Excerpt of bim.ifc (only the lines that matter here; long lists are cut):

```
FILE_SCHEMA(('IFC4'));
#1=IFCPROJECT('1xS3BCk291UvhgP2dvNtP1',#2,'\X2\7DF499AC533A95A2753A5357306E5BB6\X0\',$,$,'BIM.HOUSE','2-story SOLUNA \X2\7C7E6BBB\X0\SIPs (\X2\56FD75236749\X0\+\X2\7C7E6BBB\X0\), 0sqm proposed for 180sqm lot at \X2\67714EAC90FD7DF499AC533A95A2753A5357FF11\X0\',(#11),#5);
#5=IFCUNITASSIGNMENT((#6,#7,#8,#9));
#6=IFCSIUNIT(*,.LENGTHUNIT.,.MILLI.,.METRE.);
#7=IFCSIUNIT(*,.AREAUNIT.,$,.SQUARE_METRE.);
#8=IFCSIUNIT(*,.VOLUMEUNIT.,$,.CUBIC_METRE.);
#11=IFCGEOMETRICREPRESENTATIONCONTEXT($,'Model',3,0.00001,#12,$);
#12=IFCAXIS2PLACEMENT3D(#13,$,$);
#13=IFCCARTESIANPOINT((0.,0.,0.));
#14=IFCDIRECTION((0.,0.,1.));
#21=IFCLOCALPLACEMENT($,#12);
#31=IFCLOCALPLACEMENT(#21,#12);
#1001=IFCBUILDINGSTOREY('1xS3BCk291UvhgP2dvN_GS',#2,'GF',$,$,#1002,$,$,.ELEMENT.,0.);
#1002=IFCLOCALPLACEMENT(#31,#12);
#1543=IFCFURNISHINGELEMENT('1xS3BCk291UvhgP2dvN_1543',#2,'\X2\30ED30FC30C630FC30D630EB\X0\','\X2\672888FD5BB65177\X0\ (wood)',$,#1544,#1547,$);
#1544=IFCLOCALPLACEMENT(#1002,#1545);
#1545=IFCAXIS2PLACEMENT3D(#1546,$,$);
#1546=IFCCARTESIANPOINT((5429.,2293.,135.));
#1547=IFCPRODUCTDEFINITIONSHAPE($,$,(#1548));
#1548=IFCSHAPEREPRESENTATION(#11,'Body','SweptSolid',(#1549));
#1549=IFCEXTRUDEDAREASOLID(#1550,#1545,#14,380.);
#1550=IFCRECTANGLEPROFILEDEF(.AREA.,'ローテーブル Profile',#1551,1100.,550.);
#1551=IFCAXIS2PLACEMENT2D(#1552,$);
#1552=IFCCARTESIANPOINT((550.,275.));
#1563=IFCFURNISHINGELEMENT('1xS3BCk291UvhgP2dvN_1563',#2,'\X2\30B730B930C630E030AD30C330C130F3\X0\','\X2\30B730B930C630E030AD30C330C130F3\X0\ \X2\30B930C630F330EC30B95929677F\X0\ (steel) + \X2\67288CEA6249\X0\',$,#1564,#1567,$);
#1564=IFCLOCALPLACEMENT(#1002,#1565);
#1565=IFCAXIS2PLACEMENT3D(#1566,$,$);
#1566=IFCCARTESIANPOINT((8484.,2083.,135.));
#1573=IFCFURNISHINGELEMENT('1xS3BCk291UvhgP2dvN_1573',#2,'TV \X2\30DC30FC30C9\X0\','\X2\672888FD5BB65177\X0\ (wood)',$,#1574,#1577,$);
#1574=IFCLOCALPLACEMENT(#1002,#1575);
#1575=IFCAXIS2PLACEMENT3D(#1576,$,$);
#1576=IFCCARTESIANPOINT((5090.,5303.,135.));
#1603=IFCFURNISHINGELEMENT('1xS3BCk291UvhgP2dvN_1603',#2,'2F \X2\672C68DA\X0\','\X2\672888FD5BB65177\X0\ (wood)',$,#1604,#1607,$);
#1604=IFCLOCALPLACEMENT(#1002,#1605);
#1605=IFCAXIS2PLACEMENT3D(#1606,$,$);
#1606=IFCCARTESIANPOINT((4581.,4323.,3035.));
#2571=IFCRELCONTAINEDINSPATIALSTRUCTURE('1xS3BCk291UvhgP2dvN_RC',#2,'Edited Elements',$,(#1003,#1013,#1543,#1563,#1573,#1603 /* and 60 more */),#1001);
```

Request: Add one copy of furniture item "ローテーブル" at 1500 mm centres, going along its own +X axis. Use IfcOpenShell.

```python
import ifcopenshell
import ifcopenshell.api.geometry
import ifcopenshell.api.root
import ifcopenshell.util.element
import ifcopenshell.util.placement
import ifcopenshell.util.unit

model = ifcopenshell.open("bim.ifc")
unit_scale = ifcopenshell.util.unit.calculate_unit_scale(model)


def reuse_history(source, copy):
    """copy_class also copies each property set's owner history, people and application; keep the originals."""
    for rel in copy.IsDefinedBy:
        if rel.is_a("IfcRelDefinesByProperties") and (history := rel.RelatingPropertyDefinition.OwnerHistory):
            rel.RelatingPropertyDefinition.OwnerHistory = source.OwnerHistory
            ifcopenshell.util.element.remove_deep2(model, history)


source = model.by_guid("1xS3BCk291UvhgP2dvN_1543")
base = ifcopenshell.util.placement.get_local_placement(source.ObjectPlacement)
step = base[:3, 0] * 1.5 / unit_scale

for i in range(1, 2):
    copy = ifcopenshell.api.root.copy_class(model, product=source)
    copy.Representation = ifcopenshell.util.element.copy_deep(
        model, source.Representation, exclude=["IfcGeometricRepresentationContext", "IfcRepresentationMap"]
    )
    reuse_history(source, copy)
    matrix = base.copy()
    matrix[:3, 3] += i * step
    print("added at", matrix[:3, 3].round(3) + 0.0)
    ifcopenshell.api.geometry.edit_object_placement(model, product=copy, matrix=matrix, is_si=False)

model.write("bim_v2.ifc")
```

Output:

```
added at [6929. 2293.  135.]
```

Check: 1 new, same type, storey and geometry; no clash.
